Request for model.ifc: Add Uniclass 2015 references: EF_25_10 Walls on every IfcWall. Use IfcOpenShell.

First a look at what the model holds.

```python
import ifcopenshell

model = ifcopenshell.open("model.ifc")
print(model.schema)
print("classifications:", [c.Name for c in model.by_type("IfcClassification")])
for ifc_class in ("IfcDoor", "IfcRoof", "IfcStair", "IfcWall", "IfcWindow"):
    print(ifc_class, len(model.by_type(ifc_class)))
```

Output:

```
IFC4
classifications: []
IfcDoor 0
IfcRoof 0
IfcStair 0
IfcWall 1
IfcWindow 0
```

```python
import ifcopenshell
import ifcopenshell.api.classification

model = ifcopenshell.open("model.ifc")

system = ifcopenshell.api.classification.add_classification(model, classification="Uniclass 2015")

codes = {
    "IfcWall": ("EF_25_10", "Walls"),
}
for ifc_class, (code, name) in codes.items():
    products = model.by_type(ifc_class)
    ifcopenshell.api.classification.add_reference(
        model, products=products, classification=system, identification=code, name=name
    )
    print(code, len(products))

model.write("model_updated.ifc")
```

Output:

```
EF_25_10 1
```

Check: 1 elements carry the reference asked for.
